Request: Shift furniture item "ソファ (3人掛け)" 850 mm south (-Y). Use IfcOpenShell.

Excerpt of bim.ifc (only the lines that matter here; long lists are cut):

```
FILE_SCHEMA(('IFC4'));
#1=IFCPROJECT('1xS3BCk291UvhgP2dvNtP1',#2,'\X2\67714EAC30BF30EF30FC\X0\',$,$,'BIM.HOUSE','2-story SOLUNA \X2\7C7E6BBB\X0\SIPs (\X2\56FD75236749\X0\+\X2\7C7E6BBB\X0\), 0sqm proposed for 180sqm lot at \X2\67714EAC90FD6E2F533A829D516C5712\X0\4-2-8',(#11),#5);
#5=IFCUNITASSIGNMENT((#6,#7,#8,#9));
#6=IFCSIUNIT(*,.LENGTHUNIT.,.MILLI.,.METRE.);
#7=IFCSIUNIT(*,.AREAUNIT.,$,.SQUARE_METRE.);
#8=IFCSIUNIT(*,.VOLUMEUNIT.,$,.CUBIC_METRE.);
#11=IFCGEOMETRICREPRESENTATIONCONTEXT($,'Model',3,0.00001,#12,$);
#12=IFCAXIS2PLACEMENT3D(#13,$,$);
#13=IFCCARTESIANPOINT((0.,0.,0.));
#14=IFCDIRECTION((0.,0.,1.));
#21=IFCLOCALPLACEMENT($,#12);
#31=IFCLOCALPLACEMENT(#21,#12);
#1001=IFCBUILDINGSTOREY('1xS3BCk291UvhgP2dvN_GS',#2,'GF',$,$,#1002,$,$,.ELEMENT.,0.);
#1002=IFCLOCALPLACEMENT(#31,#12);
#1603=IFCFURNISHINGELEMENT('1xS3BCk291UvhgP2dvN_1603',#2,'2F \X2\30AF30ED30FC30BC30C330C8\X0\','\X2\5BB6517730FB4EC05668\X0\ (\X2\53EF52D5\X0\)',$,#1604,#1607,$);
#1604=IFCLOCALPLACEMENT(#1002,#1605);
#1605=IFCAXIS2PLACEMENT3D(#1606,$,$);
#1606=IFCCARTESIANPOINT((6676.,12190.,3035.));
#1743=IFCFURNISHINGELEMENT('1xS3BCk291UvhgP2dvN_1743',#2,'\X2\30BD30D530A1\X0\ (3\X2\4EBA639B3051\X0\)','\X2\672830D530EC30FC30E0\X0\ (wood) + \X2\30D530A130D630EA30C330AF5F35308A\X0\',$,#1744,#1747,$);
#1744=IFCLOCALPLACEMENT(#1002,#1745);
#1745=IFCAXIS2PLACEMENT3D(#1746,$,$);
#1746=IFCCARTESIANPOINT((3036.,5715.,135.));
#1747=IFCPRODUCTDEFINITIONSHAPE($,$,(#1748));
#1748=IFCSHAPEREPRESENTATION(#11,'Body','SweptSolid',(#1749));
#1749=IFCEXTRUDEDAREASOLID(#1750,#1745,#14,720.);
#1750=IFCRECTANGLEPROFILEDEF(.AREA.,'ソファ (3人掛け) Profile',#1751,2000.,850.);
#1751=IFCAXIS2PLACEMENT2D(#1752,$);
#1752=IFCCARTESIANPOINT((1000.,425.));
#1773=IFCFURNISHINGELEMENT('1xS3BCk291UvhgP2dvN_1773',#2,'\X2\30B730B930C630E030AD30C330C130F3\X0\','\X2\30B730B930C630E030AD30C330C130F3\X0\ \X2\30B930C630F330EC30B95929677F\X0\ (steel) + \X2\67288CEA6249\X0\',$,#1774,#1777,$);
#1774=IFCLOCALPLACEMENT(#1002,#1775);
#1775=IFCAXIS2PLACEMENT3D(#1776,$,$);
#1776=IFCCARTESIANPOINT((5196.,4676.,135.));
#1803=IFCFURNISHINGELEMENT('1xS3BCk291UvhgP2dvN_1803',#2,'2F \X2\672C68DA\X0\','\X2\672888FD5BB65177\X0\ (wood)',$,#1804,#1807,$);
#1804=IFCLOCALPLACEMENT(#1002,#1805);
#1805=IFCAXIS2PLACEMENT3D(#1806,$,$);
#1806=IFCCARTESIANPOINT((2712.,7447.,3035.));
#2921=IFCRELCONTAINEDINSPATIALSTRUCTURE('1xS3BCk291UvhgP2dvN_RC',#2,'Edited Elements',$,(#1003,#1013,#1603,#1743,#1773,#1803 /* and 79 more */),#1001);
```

```python
import ifcopenshell
import ifcopenshell.api.geometry
import ifcopenshell.util.placement
import ifcopenshell.util.unit

model = ifcopenshell.open("bim.ifc")
unit_scale = ifcopenshell.util.unit.calculate_unit_scale(model)

item = model.by_guid("1xS3BCk291UvhgP2dvN_1743")
matrix = ifcopenshell.util.placement.get_local_placement(item.ObjectPlacement)
matrix[1, 3] -= 0.85 / unit_scale
ifcopenshell.api.geometry.edit_object_placement(model, product=item, matrix=matrix, is_si=False)

print(ifcopenshell.util.placement.get_local_placement(item.ObjectPlacement).round(3) + 0.0)

model.write("bim_v2.ifc")
```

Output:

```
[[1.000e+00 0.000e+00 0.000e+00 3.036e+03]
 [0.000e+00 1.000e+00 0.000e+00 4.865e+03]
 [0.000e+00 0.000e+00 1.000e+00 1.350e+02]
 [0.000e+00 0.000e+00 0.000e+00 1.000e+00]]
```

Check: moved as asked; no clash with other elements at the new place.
